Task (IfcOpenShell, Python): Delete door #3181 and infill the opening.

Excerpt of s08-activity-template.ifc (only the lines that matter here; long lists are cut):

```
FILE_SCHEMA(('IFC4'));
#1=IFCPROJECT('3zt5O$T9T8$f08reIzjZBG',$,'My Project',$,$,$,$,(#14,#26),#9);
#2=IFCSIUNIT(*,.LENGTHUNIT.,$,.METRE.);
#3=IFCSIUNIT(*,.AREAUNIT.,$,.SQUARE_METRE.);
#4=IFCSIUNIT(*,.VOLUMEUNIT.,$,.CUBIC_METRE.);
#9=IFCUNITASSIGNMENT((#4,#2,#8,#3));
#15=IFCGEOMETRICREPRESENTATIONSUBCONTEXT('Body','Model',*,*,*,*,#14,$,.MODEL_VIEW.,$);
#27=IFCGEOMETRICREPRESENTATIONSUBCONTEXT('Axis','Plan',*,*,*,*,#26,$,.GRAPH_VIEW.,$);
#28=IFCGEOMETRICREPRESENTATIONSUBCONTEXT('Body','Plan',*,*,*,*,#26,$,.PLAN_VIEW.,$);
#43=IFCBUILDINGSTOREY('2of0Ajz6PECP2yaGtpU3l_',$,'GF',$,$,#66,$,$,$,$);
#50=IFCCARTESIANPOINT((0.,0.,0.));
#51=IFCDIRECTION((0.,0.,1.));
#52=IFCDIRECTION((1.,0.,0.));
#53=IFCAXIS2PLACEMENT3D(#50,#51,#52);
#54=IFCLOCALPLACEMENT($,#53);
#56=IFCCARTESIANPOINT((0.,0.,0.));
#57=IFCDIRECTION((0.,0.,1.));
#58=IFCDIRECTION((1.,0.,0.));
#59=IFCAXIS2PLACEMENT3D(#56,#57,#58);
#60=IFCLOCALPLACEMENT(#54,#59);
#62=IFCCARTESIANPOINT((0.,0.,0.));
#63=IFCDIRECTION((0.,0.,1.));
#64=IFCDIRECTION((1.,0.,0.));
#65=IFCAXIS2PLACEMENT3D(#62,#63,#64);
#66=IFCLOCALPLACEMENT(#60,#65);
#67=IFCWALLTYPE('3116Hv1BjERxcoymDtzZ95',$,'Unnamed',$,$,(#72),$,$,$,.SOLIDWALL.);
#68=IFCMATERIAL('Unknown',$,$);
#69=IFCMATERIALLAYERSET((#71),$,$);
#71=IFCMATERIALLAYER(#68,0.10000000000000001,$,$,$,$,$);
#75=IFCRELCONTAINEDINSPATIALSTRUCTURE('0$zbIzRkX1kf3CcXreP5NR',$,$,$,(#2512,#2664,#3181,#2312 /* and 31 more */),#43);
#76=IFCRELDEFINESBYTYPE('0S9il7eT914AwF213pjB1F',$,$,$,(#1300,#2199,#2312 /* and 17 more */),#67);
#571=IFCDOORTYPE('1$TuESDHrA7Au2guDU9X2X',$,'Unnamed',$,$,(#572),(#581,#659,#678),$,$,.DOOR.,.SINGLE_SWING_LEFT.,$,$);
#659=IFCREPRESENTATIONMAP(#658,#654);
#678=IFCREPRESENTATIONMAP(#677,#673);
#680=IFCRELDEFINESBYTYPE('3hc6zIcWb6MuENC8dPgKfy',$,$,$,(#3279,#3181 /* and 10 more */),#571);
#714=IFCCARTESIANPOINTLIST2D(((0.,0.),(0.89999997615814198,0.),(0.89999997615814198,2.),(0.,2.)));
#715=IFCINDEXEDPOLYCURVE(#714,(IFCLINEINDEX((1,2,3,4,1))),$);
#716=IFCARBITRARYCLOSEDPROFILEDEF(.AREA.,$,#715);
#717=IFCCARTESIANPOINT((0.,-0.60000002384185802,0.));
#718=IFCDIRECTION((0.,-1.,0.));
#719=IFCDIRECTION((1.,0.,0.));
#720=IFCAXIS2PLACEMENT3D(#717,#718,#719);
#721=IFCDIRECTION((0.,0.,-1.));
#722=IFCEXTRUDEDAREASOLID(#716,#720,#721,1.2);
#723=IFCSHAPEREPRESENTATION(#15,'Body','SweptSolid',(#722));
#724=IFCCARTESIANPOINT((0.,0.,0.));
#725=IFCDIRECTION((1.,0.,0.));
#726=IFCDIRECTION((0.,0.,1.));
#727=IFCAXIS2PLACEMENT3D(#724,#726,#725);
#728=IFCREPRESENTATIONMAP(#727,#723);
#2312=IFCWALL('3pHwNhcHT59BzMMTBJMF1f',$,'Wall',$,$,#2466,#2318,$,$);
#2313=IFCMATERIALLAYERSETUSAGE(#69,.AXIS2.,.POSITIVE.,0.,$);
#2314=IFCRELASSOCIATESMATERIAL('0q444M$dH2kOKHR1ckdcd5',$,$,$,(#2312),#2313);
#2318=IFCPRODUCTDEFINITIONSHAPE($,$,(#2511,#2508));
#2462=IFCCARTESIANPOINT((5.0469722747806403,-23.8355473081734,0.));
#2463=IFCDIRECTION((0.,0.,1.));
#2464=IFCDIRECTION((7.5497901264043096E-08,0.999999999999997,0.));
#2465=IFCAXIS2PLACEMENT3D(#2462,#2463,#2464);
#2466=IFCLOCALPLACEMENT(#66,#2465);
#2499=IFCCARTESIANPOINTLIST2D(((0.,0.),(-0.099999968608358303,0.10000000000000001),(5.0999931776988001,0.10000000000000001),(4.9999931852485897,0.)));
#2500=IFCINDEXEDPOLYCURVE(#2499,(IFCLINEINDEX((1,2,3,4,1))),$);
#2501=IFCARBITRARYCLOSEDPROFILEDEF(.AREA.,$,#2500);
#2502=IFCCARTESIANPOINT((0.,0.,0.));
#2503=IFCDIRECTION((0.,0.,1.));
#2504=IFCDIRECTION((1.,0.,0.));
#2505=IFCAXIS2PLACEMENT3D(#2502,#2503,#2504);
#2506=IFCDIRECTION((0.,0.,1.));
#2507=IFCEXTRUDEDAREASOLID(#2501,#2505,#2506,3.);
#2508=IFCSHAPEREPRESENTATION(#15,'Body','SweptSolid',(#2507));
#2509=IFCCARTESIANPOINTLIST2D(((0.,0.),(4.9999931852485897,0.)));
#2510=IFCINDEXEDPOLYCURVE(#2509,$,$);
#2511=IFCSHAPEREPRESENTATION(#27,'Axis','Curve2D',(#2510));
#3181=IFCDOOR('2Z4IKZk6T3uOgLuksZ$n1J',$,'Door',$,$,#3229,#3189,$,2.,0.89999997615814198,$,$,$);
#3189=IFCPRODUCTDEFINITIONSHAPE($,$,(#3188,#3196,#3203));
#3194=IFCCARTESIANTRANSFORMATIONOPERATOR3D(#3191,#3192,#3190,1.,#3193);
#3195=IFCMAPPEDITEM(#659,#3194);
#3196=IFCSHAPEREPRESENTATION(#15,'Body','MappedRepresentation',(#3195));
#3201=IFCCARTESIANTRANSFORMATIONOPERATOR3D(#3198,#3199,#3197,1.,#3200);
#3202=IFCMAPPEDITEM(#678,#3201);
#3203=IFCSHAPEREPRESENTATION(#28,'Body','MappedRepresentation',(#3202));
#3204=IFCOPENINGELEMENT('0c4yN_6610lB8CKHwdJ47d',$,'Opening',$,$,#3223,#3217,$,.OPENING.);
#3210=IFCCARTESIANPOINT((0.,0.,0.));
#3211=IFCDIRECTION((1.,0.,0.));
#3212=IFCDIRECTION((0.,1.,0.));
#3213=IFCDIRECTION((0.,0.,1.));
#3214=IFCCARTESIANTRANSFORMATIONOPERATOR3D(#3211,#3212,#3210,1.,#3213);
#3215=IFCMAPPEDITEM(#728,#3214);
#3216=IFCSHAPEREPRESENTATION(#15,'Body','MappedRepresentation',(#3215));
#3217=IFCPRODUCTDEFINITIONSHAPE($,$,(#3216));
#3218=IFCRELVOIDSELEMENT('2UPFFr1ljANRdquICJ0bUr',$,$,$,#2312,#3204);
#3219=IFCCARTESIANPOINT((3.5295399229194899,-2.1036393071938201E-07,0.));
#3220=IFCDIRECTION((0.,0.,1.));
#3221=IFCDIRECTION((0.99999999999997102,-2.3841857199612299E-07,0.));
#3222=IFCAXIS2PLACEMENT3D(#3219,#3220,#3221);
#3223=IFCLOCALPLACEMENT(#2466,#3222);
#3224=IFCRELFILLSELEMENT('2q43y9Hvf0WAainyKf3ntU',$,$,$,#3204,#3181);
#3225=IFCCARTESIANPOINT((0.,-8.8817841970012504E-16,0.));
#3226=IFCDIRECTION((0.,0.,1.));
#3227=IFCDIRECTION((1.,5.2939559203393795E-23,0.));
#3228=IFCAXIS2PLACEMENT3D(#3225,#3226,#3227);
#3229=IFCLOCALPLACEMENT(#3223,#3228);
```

```python
import ifcopenshell
import ifcopenshell.api.feature
import ifcopenshell.api.root
import ifcopenshell.geom
import ifcopenshell.util.shape

model = ifcopenshell.open("s08-activity-template.ifc")
settings = ifcopenshell.geom.settings()


def volume(element):
    """Net volume in cubic metres, openings subtracted."""
    shape = ifcopenshell.geom.create_shape(settings, element)
    return ifcopenshell.util.shape.get_volume(shape.geometry)


door = model.by_guid("2Z4IKZk6T3uOgLuksZ$n1J")
opening = door.FillsVoids[0].RelatingOpeningElement
wall = opening.VoidsElements[0].RelatingBuildingElement
before = volume(wall)

ifcopenshell.api.root.remove_product(model, product=door)
ifcopenshell.api.feature.remove_feature(model, feature=opening)

after = volume(wall)

print(f"wall volume {before:.3f} -> {after:.3f} m3")

model.write("s08-activity-template_v2.ifc")
```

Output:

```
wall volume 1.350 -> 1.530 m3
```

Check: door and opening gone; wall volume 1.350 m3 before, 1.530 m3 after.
